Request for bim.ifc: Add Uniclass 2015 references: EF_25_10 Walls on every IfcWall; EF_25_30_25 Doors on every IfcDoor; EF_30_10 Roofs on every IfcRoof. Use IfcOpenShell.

First a look at what the model holds.

```python
import ifcopenshell

model = ifcopenshell.open("bim.ifc")
print(model.schema)
print("classifications:", [c.Name for c in model.by_type("IfcClassification")])
for ifc_class in ("IfcDoor", "IfcRoof", "IfcStair", "IfcWall", "IfcWindow"):
    print(ifc_class, len(model.by_type(ifc_class)))
```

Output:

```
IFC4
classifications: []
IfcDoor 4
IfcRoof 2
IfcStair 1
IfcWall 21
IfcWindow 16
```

```python
import ifcopenshell
import ifcopenshell.api.classification

model = ifcopenshell.open("bim.ifc")

system = ifcopenshell.api.classification.add_classification(model, classification="Uniclass 2015")

codes = {
    "IfcWall": ("EF_25_10", "Walls"),
    "IfcDoor": ("EF_25_30_25", "Doors"),
    "IfcRoof": ("EF_30_10", "Roofs"),
}
for ifc_class, (code, name) in codes.items():
    products = model.by_type(ifc_class)
    ifcopenshell.api.classification.add_reference(
        model, products=products, classification=system, identification=code, name=name
    )
    print(code, len(products))

model.write("bim_updated.ifc")
```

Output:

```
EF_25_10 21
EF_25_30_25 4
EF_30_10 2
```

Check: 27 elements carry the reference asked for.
